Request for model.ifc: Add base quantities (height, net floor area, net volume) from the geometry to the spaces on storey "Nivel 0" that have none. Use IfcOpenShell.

First a look at what the model holds.

```python
import ifcopenshell
import ifcopenshell.util.element
import ifcopenshell.util.unit

model = ifcopenshell.open("model.ifc")
print(model.schema)
for unit_type in ("LENGTHUNIT", "AREAUNIT", "VOLUMEUNIT"):
    print(unit_type, ifcopenshell.util.unit.calculate_unit_scale(model, unit_type))
storey = next(s for s in model.by_type("IfcBuildingStorey") if s.Name == "Nivel 0")
spaces = [e for e in ifcopenshell.util.element.get_decomposition(storey) if e.is_a("IfcSpace")]
for e in sorted(spaces, key=lambda e: e.id()):
    print(e.id(), e.is_a(), e.Name, list(ifcopenshell.util.element.get_psets(e, qtos_only=True)), sep=" | ")
```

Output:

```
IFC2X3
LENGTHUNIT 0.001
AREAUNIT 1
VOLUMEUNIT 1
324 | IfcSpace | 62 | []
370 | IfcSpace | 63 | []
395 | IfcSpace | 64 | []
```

```python
import ifcopenshell
import ifcopenshell.api.pset
import ifcopenshell.geom
import ifcopenshell.util.element
import ifcopenshell.util.shape
import ifcopenshell.util.unit

model = ifcopenshell.open("model.ifc")
unit_scale = ifcopenshell.util.unit.calculate_unit_scale(model)
area_scale = ifcopenshell.util.unit.calculate_unit_scale(model, "AREAUNIT")
volume_scale = ifcopenshell.util.unit.calculate_unit_scale(model, "VOLUMEUNIT")
settings = ifcopenshell.geom.settings()

storey = next(s for s in model.by_type("IfcBuildingStorey") if s.Name == "Nivel 0")
spaces = [e for e in ifcopenshell.util.element.get_decomposition(storey) if e.is_a("IfcSpace")]

for e in sorted(spaces, key=lambda e: e.id()):
    if ifcopenshell.util.element.get_psets(e, qtos_only=True, should_inherit=False):
        continue
    # Geometry comes back in metres, in the element's own axes.
    shape = ifcopenshell.geom.create_shape(settings, e)
    values = {
        "Height": ifcopenshell.util.shape.get_z(shape.geometry) / unit_scale,
        "NetFloorArea": ifcopenshell.util.shape.get_footprint_area(shape.geometry) / area_scale,
        "NetVolume": ifcopenshell.util.shape.get_volume(shape.geometry) / volume_scale,
    }
    qto = ifcopenshell.api.pset.add_qto(model, product=e, name="BaseQuantities")
    ifcopenshell.api.pset.edit_qto(model, qto=qto, properties=values)
    print(e.id(), {k: round(v, 3) for k, v in values.items()})

model.write("model_v2.ifc")
```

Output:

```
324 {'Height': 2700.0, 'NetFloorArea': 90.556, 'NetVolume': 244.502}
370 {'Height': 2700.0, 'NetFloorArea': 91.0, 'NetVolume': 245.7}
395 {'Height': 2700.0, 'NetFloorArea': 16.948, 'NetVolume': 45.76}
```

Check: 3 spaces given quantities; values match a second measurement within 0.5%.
